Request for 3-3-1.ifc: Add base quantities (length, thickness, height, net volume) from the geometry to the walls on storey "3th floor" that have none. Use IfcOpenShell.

First a look at what the model holds.

```python
import ifcopenshell
import ifcopenshell.util.element
import ifcopenshell.util.unit

model = ifcopenshell.open("3-3-1.ifc")
print(model.schema)
for unit_type in ("LENGTHUNIT", "AREAUNIT", "VOLUMEUNIT"):
    print(unit_type, ifcopenshell.util.unit.calculate_unit_scale(model, unit_type))
storey = next(s for s in model.by_type("IfcBuildingStorey") if s.Name == "3th floor")
walls = [e for e in ifcopenshell.util.element.get_decomposition(storey) if e.is_a("IfcWall")]
for e in sorted(walls, key=lambda e: e.id()):
    print(e.id(), e.is_a(), e.Name, list(ifcopenshell.util.element.get_psets(e, qtos_only=True)), sep=" | ")
```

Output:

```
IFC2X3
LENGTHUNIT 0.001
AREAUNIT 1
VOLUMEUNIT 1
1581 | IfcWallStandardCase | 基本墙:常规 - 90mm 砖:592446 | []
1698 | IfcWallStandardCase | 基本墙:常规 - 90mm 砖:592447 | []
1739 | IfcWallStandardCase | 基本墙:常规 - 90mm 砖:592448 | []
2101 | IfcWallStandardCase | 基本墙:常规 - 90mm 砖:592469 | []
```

```python
import ifcopenshell
import ifcopenshell.api.pset
import ifcopenshell.geom
import ifcopenshell.util.element
import ifcopenshell.util.shape
import ifcopenshell.util.unit

model = ifcopenshell.open("3-3-1.ifc")
unit_scale = ifcopenshell.util.unit.calculate_unit_scale(model)
volume_scale = ifcopenshell.util.unit.calculate_unit_scale(model, "VOLUMEUNIT")
settings = ifcopenshell.geom.settings()

storey = next(s for s in model.by_type("IfcBuildingStorey") if s.Name == "3th floor")
walls = [e for e in ifcopenshell.util.element.get_decomposition(storey) if e.is_a("IfcWall")]

for e in sorted(walls, key=lambda e: e.id()):
    if ifcopenshell.util.element.get_psets(e, qtos_only=True, should_inherit=False):
        continue
    # Geometry comes back in metres, in the element's own axes.
    shape = ifcopenshell.geom.create_shape(settings, e)
    values = {
        "Length": ifcopenshell.util.shape.get_x(shape.geometry) / unit_scale,
        "Width": ifcopenshell.util.shape.get_y(shape.geometry) / unit_scale,
        "Height": ifcopenshell.util.shape.get_z(shape.geometry) / unit_scale,
        "NetVolume": ifcopenshell.util.shape.get_volume(shape.geometry) / volume_scale,
    }
    qto = ifcopenshell.api.pset.add_qto(model, product=e, name="BaseQuantities")
    ifcopenshell.api.pset.edit_qto(model, qto=qto, properties=values)
    print(e.id(), {k: round(v, 3) for k, v in values.items()})

model.write("3-3-1-out.ifc")
```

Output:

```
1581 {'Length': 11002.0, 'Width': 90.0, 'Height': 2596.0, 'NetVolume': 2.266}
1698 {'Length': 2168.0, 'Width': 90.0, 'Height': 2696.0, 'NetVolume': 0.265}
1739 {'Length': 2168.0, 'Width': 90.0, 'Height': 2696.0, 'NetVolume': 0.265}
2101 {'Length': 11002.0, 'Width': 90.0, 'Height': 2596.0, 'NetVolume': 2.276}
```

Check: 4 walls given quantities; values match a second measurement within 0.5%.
